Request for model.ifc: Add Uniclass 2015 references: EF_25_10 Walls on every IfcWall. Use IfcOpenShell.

First a look at what the model holds.

```python
import ifcopenshell

model = ifcopenshell.open("model.ifc")
print(model.schema)
print("classifications:", [c.Name for c in model.by_type("IfcClassification")])
for ifc_class in ("IfcDoor", "IfcRoof", "IfcStair", "IfcWall", "IfcWindow"):
    print(ifc_class, len(model.by_type(ifc_class)))
```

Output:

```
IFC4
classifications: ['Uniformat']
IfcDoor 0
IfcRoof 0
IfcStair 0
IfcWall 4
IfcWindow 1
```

```python
import ifcopenshell
import ifcopenshell.api.classification

model = ifcopenshell.open("model.ifc")

system = ifcopenshell.api.classification.add_classification(model, classification="Uniclass 2015")

codes = {
    "IfcWall": ("EF_25_10", "Walls"),
}
for ifc_class, (code, name) in codes.items():
    products = model.by_type(ifc_class)
    ifcopenshell.api.classification.add_reference(
        model, products=products, classification=system, identification=code, name=name
    )
    print(code, len(products))

model.write("model_edited.ifc")
```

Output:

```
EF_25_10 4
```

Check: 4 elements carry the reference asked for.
